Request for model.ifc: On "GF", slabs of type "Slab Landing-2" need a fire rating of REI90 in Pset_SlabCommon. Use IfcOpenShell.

First a look at what the model holds.

```python
import ifcopenshell
import ifcopenshell.util.element

model = ifcopenshell.open("model.ifc")
print(model.schema)
storey = next(s for s in model.by_type("IfcBuildingStorey") if s.Name == "GF")
slabs = [e for e in ifcopenshell.util.element.get_decomposition(storey) if e.is_a("IfcSlab")]
seen = {}
for e in slabs:
    element_type = ifcopenshell.util.element.get_type(e)
    key = (element_type.Name if element_type != e and element_type else None, ifcopenshell.util.element.get_pset(e, "Pset_SlabCommon", "FireRating"))
    seen[key] = seen.get(key, 0) + 1
for (name, value), count in sorted(seen.items(), key=str):
    print(count, "x", name, "|", value)
```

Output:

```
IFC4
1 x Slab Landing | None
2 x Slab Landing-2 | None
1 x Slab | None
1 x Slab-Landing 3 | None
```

```python
import ifcopenshell
import ifcopenshell.api.pset
import ifcopenshell.util.element

model = ifcopenshell.open("model.ifc")

storey = next(s for s in model.by_type("IfcBuildingStorey") if s.Name == "GF")
slabs = [e for e in ifcopenshell.util.element.get_decomposition(storey) if e.is_a("IfcSlab")]

count = 0
for e in slabs:
    element_type = ifcopenshell.util.element.get_type(e)
    if element_type in (None, e) or element_type.Name != "Slab Landing-2":
        continue
    # add_pset returns the element's existing set when there is one.
    pset = ifcopenshell.api.pset.add_pset(model, product=e, name="Pset_SlabCommon")
    ifcopenshell.api.pset.edit_pset(model, pset=pset, properties={"FireRating": "REI90"})
    count += 1

print(count, "slabs updated")

model.write("model-out.ifc")
```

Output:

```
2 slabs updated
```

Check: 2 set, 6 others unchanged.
